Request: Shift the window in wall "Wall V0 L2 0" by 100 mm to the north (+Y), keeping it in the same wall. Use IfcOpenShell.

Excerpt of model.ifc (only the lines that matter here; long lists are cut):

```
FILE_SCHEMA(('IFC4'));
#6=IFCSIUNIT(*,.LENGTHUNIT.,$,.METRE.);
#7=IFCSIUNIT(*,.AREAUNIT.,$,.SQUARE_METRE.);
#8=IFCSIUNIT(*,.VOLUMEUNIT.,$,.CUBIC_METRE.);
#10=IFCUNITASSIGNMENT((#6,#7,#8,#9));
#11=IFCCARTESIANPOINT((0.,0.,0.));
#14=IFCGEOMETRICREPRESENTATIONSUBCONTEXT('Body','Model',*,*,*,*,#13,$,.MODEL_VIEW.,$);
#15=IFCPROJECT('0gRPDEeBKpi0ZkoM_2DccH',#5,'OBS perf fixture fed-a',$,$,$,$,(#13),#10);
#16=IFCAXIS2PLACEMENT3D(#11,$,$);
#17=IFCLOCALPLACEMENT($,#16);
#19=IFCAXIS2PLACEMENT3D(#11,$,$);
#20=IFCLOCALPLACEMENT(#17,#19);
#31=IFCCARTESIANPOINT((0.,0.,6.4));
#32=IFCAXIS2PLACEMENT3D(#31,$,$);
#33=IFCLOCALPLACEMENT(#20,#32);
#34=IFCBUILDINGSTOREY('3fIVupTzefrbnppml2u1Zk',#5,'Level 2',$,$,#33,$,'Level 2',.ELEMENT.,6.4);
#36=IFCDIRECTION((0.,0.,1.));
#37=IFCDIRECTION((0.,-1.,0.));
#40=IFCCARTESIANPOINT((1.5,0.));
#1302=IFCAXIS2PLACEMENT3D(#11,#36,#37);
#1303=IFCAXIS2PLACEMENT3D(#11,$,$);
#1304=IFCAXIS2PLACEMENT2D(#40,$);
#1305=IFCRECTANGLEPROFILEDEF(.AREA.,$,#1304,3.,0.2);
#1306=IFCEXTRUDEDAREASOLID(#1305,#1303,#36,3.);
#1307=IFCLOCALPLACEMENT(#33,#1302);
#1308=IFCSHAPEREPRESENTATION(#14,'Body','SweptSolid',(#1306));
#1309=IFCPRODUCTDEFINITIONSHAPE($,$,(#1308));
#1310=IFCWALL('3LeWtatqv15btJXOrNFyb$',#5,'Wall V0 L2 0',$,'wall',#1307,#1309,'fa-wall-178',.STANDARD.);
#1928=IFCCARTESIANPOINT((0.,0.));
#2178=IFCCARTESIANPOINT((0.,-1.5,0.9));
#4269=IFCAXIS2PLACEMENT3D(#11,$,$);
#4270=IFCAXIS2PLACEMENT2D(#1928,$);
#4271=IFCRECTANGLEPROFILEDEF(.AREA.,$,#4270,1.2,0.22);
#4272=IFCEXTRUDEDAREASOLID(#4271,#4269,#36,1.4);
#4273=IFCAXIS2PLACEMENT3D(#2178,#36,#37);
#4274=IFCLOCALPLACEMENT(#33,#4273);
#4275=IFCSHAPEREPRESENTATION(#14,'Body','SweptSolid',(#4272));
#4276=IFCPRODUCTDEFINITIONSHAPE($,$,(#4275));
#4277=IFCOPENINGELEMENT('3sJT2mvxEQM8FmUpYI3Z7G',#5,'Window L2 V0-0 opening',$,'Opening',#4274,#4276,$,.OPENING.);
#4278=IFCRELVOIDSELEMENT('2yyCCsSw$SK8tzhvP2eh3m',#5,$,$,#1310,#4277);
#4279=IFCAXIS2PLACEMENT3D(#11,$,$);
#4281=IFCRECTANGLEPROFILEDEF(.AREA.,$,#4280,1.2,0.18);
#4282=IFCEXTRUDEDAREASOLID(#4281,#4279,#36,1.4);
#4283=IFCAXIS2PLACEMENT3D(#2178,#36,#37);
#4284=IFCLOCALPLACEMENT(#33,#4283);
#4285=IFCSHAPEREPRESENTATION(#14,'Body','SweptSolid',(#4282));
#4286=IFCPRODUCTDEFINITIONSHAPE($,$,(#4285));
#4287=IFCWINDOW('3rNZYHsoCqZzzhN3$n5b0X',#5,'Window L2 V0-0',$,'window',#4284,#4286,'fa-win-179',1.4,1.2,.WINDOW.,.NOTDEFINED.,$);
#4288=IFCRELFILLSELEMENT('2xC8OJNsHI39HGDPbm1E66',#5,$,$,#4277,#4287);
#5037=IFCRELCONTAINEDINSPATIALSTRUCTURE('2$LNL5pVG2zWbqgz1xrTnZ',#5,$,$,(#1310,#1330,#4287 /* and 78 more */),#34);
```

```python
import ifcopenshell
import ifcopenshell.api.geometry
import ifcopenshell.util.placement
import ifcopenshell.util.unit

model = ifcopenshell.open("model.ifc")
unit_scale = ifcopenshell.util.unit.calculate_unit_scale(model)

window = model.by_guid("3rNZYHsoCqZzzhN3$n5b0X")
opening = window.FillsVoids[0].RelatingOpeningElement
wall = opening.VoidsElements[0].RelatingBuildingElement

wall_matrix = ifcopenshell.util.placement.get_local_placement(wall.ObjectPlacement)
shift = wall_matrix[:3, 0] * -0.1 / unit_scale
before = ifcopenshell.util.placement.get_local_placement(window.ObjectPlacement)[:3, 3].copy()

# The window is not placed relative to its opening, so move both.
for product in (opening, window):
    matrix = ifcopenshell.util.placement.get_local_placement(product.ObjectPlacement)
    matrix[:3, 3] += shift
    ifcopenshell.api.geometry.edit_object_placement(model, product=product, matrix=matrix, is_si=False)

after = ifcopenshell.util.placement.get_local_placement(window.ObjectPlacement)[:3, 3]
print("window moved by", (after - before).round(3) + 0.0)

model.write("model_rev.ifc")
```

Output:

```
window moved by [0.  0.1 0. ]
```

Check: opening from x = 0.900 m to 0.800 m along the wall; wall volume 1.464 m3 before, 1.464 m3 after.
